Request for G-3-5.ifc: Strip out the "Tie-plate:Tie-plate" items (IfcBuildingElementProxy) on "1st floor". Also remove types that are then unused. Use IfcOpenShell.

First a look at what the model holds.

```python
import ifcopenshell
import ifcopenshell.util.element

model = ifcopenshell.open("G-3-5.ifc")
print(model.schema)
storey = next(s for s in model.by_type("IfcBuildingStorey") if s.Name == "1st floor")
proxies = [e for e in ifcopenshell.util.element.get_decomposition(storey) if e.is_a("IfcBuildingElementProxy")]
seen = {}
for e in proxies:
    element_type = ifcopenshell.util.element.get_type(e)
    name = element_type.Name if element_type not in (None, e) else None
    seen[name] = seen.get(name, 0) + 1
for name, count in sorted(seen.items(), key=str):
    print(count, "x", name)
```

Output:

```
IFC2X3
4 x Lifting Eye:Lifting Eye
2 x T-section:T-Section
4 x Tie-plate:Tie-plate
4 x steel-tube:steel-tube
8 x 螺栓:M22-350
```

```python
import ifcopenshell
import ifcopenshell.api.root
import ifcopenshell.util.element

model = ifcopenshell.open("G-3-5.ifc")

storey = next(s for s in model.by_type("IfcBuildingStorey") if s.Name == "1st floor")
proxies = [e for e in ifcopenshell.util.element.get_decomposition(storey) if e.is_a("IfcBuildingElementProxy")]
targets = [e for e in proxies if (t := ifcopenshell.util.element.get_type(e)) not in (None, e) and t.Name == "Tie-plate:Tie-plate"]
types = {ifcopenshell.util.element.get_type(e) for e in targets} - {None, *targets}

for e in targets:
    ifcopenshell.api.root.remove_product(model, product=e)
print(len(targets), "removed")

unused = [t for t in types if not ifcopenshell.util.element.get_types(t)]
for t in unused:
    ifcopenshell.api.root.remove_product(model, product=t)
print(len(unused), "unused types removed")

model.write("G-3-5_edited.ifc")
```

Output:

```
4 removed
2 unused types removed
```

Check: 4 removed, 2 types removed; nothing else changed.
